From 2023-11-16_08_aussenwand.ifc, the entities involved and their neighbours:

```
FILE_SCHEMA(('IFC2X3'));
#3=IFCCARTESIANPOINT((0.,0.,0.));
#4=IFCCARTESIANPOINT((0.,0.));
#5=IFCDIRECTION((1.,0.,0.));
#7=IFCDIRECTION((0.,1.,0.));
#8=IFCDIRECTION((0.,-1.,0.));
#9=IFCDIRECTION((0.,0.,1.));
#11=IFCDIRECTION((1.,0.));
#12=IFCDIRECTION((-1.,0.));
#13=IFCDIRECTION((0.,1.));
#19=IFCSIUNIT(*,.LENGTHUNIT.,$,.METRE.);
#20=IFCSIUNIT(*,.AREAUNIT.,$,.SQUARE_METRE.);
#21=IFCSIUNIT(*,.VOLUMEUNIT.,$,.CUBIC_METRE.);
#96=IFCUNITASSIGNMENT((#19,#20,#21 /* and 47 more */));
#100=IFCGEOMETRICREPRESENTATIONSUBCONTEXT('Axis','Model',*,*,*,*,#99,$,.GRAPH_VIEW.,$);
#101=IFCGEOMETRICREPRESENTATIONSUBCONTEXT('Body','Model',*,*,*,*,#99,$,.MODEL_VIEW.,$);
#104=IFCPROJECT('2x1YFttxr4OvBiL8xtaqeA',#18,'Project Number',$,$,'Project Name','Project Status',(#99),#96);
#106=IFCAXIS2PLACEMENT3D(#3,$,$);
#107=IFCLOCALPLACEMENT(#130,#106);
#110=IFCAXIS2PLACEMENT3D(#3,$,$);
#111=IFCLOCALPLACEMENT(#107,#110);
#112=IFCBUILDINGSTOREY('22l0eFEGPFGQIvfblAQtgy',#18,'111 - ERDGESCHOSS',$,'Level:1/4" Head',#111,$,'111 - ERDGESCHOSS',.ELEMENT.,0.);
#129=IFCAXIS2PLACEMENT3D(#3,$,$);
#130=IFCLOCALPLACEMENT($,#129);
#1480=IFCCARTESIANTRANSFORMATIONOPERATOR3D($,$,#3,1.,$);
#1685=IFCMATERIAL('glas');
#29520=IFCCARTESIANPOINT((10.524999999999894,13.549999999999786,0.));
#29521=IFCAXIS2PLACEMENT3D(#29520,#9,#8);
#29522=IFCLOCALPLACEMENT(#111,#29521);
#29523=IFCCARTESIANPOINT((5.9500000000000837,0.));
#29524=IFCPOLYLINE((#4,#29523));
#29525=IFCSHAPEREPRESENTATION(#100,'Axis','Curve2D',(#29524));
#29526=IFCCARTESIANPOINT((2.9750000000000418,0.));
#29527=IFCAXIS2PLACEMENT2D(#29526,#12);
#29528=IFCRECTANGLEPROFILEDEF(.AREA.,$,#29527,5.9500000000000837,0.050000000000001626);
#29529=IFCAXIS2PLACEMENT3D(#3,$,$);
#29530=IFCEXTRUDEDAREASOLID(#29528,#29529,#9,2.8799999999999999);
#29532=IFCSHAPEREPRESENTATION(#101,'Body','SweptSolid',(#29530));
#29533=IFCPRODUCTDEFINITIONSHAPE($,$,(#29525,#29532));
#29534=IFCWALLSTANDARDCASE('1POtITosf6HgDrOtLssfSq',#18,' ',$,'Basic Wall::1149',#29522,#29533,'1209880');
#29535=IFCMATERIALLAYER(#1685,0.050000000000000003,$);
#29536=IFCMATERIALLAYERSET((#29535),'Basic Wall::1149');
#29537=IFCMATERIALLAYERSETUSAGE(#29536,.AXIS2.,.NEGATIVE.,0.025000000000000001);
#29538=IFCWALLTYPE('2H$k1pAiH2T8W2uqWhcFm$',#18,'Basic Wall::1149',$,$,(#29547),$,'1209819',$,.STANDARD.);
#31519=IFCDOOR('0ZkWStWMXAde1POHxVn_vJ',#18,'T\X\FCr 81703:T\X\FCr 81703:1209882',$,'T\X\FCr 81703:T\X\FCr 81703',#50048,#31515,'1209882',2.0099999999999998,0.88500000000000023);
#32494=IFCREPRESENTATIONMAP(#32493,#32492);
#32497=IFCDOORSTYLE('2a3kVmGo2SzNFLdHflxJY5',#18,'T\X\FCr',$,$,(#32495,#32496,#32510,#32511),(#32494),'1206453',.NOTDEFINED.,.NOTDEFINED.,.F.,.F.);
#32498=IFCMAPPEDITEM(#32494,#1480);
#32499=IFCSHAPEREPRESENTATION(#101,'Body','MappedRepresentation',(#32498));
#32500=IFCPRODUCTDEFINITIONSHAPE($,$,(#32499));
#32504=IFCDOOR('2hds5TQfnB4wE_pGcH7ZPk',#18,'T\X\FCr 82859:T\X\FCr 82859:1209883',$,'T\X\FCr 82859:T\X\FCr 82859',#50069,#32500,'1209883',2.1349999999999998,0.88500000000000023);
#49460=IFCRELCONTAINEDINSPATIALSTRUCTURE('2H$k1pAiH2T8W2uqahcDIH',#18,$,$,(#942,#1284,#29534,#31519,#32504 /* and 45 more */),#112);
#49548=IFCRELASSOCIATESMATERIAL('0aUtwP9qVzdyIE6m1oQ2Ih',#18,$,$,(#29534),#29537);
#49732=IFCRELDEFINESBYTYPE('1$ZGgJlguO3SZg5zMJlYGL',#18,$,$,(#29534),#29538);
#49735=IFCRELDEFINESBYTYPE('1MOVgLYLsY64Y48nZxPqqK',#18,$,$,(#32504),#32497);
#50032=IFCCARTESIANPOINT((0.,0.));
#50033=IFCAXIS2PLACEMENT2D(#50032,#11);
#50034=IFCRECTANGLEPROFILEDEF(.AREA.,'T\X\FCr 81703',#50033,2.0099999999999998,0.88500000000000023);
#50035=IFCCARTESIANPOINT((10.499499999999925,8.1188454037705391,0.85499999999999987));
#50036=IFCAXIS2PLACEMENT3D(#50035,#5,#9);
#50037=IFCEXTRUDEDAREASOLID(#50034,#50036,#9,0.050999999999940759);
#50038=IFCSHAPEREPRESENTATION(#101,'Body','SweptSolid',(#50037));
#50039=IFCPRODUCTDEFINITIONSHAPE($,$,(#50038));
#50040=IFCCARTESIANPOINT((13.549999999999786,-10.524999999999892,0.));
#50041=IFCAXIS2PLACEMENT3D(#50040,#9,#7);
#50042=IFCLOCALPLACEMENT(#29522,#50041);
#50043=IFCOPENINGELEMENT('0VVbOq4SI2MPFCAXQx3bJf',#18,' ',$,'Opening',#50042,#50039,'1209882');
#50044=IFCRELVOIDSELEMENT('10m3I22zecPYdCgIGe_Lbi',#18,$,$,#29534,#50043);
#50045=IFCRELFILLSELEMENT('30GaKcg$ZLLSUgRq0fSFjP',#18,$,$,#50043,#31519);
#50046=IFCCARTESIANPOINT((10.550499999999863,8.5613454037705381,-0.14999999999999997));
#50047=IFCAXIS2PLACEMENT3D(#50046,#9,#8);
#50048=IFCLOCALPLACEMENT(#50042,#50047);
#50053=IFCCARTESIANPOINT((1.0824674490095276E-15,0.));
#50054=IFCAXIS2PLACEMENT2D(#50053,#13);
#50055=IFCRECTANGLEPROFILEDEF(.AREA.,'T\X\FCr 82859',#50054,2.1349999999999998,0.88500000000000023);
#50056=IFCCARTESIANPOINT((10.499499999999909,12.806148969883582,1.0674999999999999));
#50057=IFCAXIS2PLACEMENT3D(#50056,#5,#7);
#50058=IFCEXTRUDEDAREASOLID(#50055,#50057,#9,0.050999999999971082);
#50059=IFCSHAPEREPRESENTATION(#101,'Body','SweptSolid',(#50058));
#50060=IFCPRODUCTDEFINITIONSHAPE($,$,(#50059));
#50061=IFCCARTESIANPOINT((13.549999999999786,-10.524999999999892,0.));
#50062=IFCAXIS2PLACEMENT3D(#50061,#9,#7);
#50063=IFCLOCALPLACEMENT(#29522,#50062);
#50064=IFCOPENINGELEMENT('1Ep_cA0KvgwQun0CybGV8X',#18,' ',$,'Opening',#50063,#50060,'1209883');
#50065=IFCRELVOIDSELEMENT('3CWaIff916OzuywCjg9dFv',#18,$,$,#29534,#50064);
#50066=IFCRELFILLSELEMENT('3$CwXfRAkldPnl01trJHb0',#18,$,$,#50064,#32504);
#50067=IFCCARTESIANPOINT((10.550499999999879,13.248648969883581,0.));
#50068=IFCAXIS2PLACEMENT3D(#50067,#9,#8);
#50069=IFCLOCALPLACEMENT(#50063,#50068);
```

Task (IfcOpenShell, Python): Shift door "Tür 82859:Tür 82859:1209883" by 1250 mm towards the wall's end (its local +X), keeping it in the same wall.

```python
import ifcopenshell
import ifcopenshell.api.geometry
import ifcopenshell.util.placement
import ifcopenshell.util.unit

model = ifcopenshell.open("2023-11-16_08_aussenwand.ifc")
unit_scale = ifcopenshell.util.unit.calculate_unit_scale(model)

door = model.by_guid("2hds5TQfnB4wE_pGcH7ZPk")
opening = door.FillsVoids[0].RelatingOpeningElement
wall = opening.VoidsElements[0].RelatingBuildingElement

wall_matrix = ifcopenshell.util.placement.get_local_placement(wall.ObjectPlacement)
shift = wall_matrix[:3, 0] * 1.25 / unit_scale
before = ifcopenshell.util.placement.get_local_placement(door.ObjectPlacement)[:3, 3].copy()

# The door is placed relative to its opening, so it follows when the opening moves.
matrix = ifcopenshell.util.placement.get_local_placement(opening.ObjectPlacement)
matrix[:3, 3] += shift
ifcopenshell.api.geometry.edit_object_placement(
    model, product=opening, matrix=matrix, is_si=False, should_transform_children=True
)

after = ifcopenshell.util.placement.get_local_placement(door.ObjectPlacement)[:3, 3]
print("door moved by", (after - before).round(3) + 0.0)

model.write("2023-11-16_08_aussenwand_rev.ifc")
```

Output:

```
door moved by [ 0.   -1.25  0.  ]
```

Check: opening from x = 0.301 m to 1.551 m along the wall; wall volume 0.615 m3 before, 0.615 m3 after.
